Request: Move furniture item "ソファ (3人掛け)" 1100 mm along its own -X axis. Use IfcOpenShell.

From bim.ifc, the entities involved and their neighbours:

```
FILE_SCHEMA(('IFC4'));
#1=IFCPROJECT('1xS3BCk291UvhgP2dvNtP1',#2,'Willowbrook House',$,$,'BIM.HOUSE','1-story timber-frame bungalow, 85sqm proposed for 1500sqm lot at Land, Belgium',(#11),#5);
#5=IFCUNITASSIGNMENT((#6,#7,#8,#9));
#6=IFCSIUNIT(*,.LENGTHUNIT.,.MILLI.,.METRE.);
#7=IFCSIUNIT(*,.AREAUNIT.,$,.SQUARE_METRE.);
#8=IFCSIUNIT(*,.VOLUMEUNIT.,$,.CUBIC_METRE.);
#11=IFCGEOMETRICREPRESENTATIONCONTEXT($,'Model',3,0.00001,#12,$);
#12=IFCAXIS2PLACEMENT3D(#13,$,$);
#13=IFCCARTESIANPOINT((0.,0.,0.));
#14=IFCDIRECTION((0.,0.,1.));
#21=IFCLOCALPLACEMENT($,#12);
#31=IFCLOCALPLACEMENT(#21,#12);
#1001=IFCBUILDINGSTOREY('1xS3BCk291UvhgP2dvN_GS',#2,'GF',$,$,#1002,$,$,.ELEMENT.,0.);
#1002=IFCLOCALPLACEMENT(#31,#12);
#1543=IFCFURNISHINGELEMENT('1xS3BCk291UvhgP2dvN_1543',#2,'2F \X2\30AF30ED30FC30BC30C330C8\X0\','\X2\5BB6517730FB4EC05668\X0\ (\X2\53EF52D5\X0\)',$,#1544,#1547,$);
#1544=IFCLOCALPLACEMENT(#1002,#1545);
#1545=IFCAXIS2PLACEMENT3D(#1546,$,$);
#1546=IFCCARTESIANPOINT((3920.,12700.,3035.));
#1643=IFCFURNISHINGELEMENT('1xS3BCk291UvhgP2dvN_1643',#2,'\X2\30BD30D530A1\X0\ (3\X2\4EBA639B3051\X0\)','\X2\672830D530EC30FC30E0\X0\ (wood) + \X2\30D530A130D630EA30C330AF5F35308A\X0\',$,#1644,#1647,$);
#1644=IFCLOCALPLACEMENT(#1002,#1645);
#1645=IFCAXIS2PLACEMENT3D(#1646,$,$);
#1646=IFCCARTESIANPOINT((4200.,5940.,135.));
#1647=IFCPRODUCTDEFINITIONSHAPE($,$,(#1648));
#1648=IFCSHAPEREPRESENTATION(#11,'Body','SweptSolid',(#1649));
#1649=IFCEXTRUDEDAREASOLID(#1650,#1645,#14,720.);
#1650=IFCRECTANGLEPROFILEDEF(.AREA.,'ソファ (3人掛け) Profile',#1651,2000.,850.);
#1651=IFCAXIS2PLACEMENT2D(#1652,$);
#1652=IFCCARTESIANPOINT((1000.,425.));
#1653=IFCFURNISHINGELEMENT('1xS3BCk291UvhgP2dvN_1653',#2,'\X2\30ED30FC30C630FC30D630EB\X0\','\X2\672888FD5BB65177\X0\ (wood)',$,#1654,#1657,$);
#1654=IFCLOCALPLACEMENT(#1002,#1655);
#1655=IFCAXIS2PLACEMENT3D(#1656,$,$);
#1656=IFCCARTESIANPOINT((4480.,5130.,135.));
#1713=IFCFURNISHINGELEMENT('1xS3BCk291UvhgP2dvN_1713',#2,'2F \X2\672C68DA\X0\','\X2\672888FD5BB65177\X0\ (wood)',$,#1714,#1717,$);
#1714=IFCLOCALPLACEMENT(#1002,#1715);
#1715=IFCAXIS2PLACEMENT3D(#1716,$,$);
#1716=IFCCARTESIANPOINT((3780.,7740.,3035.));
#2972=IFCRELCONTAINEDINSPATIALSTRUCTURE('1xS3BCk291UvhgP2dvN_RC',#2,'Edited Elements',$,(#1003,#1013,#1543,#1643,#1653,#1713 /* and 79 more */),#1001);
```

```python
import ifcopenshell
import ifcopenshell.api.geometry
import ifcopenshell.util.placement

model = ifcopenshell.open("bim.ifc")

item = model.by_guid("1xS3BCk291UvhgP2dvN_1643")
matrix = ifcopenshell.util.placement.get_local_placement(item.ObjectPlacement)
matrix[:3, 3] -= matrix[:3, 0] * 1100.0
ifcopenshell.api.geometry.edit_object_placement(model, product=item, matrix=matrix, is_si=False)

print(ifcopenshell.util.placement.get_local_placement(item.ObjectPlacement).round(3) + 0.0)

model.write("bim_updated.ifc")
```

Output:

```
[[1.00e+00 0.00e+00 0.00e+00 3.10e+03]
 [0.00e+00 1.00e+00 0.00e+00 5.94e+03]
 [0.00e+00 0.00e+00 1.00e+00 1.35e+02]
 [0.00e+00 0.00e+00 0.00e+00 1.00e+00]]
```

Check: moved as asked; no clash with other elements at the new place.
